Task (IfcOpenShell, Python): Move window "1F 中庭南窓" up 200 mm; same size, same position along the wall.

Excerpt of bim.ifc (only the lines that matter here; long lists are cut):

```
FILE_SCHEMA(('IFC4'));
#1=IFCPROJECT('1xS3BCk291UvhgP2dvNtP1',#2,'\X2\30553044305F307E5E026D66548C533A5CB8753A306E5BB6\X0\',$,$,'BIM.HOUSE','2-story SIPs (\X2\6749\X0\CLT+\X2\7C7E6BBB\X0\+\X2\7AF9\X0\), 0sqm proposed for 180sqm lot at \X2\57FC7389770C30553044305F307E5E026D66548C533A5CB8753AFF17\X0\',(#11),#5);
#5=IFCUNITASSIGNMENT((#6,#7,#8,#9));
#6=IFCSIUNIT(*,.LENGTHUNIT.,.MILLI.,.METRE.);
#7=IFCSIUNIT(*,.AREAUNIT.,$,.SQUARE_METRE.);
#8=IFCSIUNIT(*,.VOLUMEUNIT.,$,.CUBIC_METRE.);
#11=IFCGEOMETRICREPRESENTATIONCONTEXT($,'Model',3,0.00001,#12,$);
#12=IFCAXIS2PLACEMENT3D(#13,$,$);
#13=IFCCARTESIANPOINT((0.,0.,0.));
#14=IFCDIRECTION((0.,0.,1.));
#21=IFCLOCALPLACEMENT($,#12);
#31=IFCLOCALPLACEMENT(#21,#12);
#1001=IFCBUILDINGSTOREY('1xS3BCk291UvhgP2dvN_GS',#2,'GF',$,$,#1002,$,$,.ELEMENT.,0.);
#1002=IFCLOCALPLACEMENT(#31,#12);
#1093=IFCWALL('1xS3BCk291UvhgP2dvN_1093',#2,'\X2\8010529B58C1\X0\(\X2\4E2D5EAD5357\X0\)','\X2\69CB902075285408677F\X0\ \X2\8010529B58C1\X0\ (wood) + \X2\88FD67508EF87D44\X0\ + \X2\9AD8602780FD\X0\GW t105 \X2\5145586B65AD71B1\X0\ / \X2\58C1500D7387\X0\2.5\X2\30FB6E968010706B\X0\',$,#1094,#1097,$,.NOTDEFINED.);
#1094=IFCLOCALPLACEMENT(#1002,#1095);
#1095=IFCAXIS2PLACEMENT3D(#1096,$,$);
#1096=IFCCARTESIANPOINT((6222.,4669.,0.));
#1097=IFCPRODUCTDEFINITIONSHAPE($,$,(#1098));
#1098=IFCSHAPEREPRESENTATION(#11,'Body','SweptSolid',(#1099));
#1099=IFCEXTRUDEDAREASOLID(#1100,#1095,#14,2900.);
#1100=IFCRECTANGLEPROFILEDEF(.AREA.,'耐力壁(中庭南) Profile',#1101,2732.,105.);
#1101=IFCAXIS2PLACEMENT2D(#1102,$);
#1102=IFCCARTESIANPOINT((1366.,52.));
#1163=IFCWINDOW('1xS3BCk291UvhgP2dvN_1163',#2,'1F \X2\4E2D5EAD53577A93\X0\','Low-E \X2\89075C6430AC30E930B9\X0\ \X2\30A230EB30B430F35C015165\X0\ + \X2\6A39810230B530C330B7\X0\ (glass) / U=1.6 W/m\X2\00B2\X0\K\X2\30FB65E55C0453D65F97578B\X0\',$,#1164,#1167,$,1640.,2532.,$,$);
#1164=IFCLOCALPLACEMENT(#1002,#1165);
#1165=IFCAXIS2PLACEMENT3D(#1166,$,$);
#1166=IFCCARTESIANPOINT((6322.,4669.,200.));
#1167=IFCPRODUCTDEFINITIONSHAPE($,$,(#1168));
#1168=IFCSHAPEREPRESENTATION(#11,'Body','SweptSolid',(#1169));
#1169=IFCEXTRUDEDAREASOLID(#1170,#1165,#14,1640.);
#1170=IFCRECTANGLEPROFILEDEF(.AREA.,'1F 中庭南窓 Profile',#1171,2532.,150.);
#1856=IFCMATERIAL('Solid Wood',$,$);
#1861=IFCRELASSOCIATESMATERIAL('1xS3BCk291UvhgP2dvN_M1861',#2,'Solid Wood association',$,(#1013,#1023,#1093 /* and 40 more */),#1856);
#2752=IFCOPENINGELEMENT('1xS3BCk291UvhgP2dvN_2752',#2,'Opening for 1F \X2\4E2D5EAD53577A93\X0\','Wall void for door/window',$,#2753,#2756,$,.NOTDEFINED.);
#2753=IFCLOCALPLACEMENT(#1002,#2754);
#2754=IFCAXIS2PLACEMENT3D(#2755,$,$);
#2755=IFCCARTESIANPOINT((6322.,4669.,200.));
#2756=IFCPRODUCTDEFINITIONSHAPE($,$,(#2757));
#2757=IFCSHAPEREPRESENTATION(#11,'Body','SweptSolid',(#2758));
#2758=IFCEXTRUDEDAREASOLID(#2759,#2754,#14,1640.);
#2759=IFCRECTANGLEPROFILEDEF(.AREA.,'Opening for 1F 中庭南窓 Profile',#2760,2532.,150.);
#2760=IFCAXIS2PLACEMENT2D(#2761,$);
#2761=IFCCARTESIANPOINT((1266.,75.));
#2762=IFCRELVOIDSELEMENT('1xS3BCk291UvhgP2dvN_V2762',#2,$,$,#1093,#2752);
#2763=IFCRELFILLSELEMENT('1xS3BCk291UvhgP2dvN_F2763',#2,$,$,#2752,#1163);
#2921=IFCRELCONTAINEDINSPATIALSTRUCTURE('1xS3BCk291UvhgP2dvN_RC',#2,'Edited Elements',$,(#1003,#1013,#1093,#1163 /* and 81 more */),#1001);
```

```python
import numpy as np
import ifcopenshell
import ifcopenshell.api.geometry
import ifcopenshell.util.placement
import ifcopenshell.util.unit

model = ifcopenshell.open("bim.ifc")
unit_scale = ifcopenshell.util.unit.calculate_unit_scale(model)

window = model.by_guid("1xS3BCk291UvhgP2dvN_1163")
opening = window.FillsVoids[0].RelatingOpeningElement
dz = 0.2 / unit_scale

shift = np.array([0.0, 0.0, dz])
# The window is not placed relative to its opening, so move both.
for product in (opening, window):
    matrix = ifcopenshell.util.placement.get_local_placement(product.ObjectPlacement)
    matrix[:3, 3] += shift
    ifcopenshell.api.geometry.edit_object_placement(model, product=product, matrix=matrix, is_si=False)

print(f"moved by {dz * unit_scale:+.3f} m")

model.write("bim_rev.ifc")
```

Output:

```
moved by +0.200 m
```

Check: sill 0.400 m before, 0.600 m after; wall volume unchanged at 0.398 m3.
